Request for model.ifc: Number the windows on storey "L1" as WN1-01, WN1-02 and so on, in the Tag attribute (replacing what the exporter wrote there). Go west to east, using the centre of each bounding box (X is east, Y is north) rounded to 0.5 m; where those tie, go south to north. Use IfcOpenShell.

First a look at what the model holds.

```python
import ifcopenshell
import ifcopenshell.util.element
import ifcopenshell.util.placement

model = ifcopenshell.open("model.ifc")
print(model.schema)
storey = next(s for s in model.by_type("IfcBuildingStorey") if s.Name == "L1")
windows = [e for e in ifcopenshell.util.element.get_decomposition(storey) if e.is_a("IfcWindow")]
for e in sorted(windows, key=lambda e: e.id()):
    origin = ifcopenshell.util.placement.get_local_placement(e.ObjectPlacement)[:3, 3]
    print(e.id(), e.Tag, e.Name, origin.round(2) + 0.0, sep=" | ")
```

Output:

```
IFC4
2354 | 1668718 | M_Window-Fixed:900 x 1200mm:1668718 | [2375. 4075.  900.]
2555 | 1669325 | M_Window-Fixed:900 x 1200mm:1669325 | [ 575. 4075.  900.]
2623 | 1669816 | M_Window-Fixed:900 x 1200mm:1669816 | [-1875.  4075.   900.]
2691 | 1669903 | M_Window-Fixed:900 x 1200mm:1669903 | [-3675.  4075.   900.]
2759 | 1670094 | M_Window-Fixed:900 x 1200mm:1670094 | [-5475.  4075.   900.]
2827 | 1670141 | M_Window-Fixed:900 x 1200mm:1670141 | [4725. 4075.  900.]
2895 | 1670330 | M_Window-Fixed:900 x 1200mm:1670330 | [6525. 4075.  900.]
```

```python
import ifcopenshell
import ifcopenshell.geom
import ifcopenshell.util.element
import ifcopenshell.util.shape

model = ifcopenshell.open("model.ifc")
settings = ifcopenshell.geom.settings()
settings.set("use-world-coords", True)


def centre(element):
    shape = ifcopenshell.geom.create_shape(settings, element)
    return ifcopenshell.util.shape.get_bbox_centroid(shape.geometry)


storey = next(s for s in model.by_type("IfcBuildingStorey") if s.Name == "L1")
windows = [e for e in ifcopenshell.util.element.get_decomposition(storey) if e.is_a("IfcWindow")]

# Insertion points can sit at a corner or the storey origin, so sort by the geometry (in metres).
centres = {e: centre(e) for e in windows}
windows.sort(key=lambda e: (round(centres[e][0] / 0.5), centres[e][1]))

for i, e in enumerate(windows, start=1):
    number = f"WN1-{i:02d}"
    e.Tag = number
    print(e.id(), number)

model.write("model_updated.ifc")
```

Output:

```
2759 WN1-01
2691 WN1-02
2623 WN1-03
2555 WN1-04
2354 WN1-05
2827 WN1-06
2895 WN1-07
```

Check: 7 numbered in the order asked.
